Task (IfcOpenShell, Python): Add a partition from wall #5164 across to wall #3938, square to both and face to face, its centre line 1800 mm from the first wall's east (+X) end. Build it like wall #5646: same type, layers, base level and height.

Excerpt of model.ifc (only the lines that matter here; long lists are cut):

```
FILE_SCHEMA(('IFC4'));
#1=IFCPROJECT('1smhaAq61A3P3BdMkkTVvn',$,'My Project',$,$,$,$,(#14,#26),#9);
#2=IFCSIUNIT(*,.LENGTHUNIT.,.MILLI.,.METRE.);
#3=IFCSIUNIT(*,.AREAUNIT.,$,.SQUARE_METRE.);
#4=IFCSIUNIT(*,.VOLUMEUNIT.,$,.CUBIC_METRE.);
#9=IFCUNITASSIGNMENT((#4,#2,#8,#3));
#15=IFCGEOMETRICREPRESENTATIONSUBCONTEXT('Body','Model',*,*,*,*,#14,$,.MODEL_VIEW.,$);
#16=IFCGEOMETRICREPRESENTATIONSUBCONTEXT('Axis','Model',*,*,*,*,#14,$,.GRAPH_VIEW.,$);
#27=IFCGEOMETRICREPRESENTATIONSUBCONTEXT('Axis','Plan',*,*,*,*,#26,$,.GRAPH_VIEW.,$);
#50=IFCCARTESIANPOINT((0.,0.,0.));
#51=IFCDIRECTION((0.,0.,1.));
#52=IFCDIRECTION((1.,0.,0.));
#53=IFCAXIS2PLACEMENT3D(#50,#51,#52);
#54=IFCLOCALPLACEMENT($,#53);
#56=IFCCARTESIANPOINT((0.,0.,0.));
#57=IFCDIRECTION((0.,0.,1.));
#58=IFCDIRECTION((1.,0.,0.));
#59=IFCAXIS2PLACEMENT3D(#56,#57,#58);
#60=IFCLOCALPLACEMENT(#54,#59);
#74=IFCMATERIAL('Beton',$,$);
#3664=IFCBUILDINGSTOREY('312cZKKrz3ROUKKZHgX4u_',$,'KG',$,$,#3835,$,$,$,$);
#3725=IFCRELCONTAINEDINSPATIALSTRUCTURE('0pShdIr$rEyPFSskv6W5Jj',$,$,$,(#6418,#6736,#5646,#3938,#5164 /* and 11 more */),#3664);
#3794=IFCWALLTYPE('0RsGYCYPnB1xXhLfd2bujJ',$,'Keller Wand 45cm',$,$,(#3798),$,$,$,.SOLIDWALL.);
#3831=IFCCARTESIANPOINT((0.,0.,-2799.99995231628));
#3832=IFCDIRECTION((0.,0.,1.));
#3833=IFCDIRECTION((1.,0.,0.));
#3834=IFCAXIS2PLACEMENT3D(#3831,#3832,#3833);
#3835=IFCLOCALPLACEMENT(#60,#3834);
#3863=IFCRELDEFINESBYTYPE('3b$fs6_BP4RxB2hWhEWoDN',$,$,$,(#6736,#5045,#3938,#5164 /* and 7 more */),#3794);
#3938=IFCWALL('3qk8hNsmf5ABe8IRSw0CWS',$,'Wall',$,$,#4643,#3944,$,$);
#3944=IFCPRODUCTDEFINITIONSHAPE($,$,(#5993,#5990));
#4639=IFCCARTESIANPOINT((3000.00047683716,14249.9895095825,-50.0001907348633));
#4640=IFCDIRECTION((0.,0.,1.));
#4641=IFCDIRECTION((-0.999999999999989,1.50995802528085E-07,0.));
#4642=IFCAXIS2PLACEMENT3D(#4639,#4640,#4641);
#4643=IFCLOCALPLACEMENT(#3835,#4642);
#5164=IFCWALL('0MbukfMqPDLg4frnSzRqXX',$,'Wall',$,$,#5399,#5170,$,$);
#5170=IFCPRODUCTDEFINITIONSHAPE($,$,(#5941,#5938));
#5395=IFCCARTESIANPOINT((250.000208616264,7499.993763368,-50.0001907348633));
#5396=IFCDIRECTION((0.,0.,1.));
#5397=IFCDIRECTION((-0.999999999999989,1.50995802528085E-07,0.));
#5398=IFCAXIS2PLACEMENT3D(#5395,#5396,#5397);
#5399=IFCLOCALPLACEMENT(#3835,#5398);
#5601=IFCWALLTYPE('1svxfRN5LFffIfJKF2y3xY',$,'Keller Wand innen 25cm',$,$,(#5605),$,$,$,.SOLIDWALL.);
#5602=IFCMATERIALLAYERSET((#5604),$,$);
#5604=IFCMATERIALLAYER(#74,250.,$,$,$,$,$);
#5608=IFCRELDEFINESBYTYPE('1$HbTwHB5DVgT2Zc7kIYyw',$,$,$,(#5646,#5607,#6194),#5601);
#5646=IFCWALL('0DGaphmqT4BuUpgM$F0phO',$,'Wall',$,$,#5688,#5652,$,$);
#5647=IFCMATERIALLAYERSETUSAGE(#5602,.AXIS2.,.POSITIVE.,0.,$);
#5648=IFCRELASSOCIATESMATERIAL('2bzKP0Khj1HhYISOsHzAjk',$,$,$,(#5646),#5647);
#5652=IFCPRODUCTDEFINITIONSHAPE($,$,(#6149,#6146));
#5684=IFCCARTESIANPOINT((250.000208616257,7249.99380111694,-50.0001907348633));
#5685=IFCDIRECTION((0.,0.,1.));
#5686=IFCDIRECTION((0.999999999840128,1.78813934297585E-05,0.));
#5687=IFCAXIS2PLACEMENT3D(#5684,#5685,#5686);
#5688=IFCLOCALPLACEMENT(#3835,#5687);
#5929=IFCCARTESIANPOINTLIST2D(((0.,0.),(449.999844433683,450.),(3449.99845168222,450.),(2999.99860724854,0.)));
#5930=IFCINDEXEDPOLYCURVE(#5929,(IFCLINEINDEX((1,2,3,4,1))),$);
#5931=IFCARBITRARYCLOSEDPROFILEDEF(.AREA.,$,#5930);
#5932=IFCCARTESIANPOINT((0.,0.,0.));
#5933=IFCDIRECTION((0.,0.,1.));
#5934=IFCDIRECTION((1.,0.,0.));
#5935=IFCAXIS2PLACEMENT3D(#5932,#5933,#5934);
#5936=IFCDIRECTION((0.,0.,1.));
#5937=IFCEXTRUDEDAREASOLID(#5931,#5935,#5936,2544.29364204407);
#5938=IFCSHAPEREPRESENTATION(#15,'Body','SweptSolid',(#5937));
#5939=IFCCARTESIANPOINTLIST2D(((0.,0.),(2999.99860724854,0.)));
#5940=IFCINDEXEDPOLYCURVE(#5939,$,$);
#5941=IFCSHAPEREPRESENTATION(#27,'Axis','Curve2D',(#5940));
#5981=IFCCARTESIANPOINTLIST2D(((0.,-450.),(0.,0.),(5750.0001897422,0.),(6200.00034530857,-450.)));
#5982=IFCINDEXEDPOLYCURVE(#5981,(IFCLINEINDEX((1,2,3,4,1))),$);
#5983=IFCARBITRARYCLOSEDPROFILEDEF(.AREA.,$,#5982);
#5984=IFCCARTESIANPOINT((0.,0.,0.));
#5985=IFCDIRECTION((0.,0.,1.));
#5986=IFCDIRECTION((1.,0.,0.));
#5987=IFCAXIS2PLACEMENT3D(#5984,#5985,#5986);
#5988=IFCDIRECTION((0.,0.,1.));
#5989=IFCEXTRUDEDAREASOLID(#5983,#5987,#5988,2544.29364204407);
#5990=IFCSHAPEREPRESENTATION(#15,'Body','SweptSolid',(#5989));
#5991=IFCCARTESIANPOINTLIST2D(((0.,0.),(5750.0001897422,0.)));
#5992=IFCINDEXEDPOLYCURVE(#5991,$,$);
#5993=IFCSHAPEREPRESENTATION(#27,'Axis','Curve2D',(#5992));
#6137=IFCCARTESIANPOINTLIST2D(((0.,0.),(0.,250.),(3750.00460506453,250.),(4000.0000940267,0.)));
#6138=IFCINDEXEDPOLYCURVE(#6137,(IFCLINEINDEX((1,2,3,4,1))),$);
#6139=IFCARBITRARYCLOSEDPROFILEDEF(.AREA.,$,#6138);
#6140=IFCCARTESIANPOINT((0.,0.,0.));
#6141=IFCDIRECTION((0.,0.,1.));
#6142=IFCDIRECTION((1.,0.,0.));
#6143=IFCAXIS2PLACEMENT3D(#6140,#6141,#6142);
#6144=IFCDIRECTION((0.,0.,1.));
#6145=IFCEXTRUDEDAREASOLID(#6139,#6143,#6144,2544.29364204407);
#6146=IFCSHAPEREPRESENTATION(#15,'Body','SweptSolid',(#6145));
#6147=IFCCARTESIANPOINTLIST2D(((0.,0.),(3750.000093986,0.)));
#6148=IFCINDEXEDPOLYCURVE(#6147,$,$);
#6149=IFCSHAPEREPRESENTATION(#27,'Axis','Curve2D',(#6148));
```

```python
import numpy as np
import ifcopenshell
import ifcopenshell.api.geometry
import ifcopenshell.api.material
import ifcopenshell.api.pset
import ifcopenshell.api.root
import ifcopenshell.api.spatial
import ifcopenshell.api.type
import ifcopenshell.geom
import ifcopenshell.util.element
import ifcopenshell.util.placement
import ifcopenshell.util.representation
import ifcopenshell.util.shape
import ifcopenshell.util.unit

model = ifcopenshell.open("model.ifc")
unit_scale = ifcopenshell.util.unit.calculate_unit_scale(model)
settings = ifcopenshell.geom.settings()
settings.set("use-world-coords", True)

start_wall = model.by_guid("0MbukfMqPDLg4frnSzRqXX")
end_wall = model.by_guid("3qk8hNsmf5ABe8IRSw0CWS")
like = model.by_guid("0DGaphmqT4BuUpgM$F0phO")
matrix = ifcopenshell.util.placement.get_local_placement(start_wall.ObjectPlacement)
matrix[:3, 3] *= unit_scale


def extent(element):
    """Bounding box in the first wall's axes, in metres."""
    shape = ifcopenshell.geom.create_shape(settings, element)
    points = (ifcopenshell.util.shape.get_vertices(shape.geometry) - matrix[:3, 3]) @ matrix[:3, :3]
    return points.min(axis=0), points.max(axis=0)


y_start = extent(start_wall)[0][1]
y_end = extent(end_wall)[1][1]
like_min, like_max = extent(like)
length, height = float(abs(y_end - y_start)), float(like_max[2] - like_min[2])
layer_set = ifcopenshell.util.element.get_material(like, should_skip_usage=True)
thickness = sum(layer.LayerThickness for layer in layer_set.MaterialLayers) * unit_scale

wall = ifcopenshell.api.root.create_entity(model, ifc_class="IfcWall", name="New partition")
storey = ifcopenshell.util.element.get_container(like)
ifcopenshell.api.spatial.assign_container(model, products=[wall], relating_structure=storey)
ifcopenshell.api.type.assign_type(
    model, related_objects=[wall], relating_type=ifcopenshell.util.element.get_type(like), should_map_representations=False
)
rel = ifcopenshell.api.material.assign_material(
    model, products=[wall], type="IfcMaterialLayerSetUsage", material=layer_set
)
rel.RelatingMaterial.OffsetFromReferenceLine = -thickness / 2 / unit_scale
pset = ifcopenshell.api.pset.add_pset(model, product=wall, name="Pset_WallCommon")
ifcopenshell.api.pset.edit_pset(model, pset=pset, properties={"IsExternal": False, "LoadBearing": False})

# The axis runs down the middle of the wall.
axis = ifcopenshell.api.geometry.add_axis_representation(
    model, context=ifcopenshell.util.representation.get_context(model, "Model", "Axis"), axis=[(0.0, 0.0), (length, 0.0)]
)
body = ifcopenshell.api.geometry.add_wall_representation(
    model,
    context=ifcopenshell.util.representation.get_context(model, "Model", "Body", "MODEL_VIEW"),
    length=length,
    height=height,
    thickness=thickness,
    offset=-thickness / 2,
)
for representation in (axis, body):
    ifcopenshell.api.geometry.assign_representation(model, product=wall, representation=representation)

placement = matrix @ ifcopenshell.util.placement.rotation(-90, "Z")
placement[:, 3] = matrix @ np.array([extent(start_wall)[0][0] + 1.8, y_start, like_min[2], 1.0])
ifcopenshell.api.geometry.edit_object_placement(model, product=wall, matrix=placement)

print(f"partition {length:.3f} m long, {height:.3f} m high, {thickness:.3f} m thick")

model.write("model-out.ifc")
```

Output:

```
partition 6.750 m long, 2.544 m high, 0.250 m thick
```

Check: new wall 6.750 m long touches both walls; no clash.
